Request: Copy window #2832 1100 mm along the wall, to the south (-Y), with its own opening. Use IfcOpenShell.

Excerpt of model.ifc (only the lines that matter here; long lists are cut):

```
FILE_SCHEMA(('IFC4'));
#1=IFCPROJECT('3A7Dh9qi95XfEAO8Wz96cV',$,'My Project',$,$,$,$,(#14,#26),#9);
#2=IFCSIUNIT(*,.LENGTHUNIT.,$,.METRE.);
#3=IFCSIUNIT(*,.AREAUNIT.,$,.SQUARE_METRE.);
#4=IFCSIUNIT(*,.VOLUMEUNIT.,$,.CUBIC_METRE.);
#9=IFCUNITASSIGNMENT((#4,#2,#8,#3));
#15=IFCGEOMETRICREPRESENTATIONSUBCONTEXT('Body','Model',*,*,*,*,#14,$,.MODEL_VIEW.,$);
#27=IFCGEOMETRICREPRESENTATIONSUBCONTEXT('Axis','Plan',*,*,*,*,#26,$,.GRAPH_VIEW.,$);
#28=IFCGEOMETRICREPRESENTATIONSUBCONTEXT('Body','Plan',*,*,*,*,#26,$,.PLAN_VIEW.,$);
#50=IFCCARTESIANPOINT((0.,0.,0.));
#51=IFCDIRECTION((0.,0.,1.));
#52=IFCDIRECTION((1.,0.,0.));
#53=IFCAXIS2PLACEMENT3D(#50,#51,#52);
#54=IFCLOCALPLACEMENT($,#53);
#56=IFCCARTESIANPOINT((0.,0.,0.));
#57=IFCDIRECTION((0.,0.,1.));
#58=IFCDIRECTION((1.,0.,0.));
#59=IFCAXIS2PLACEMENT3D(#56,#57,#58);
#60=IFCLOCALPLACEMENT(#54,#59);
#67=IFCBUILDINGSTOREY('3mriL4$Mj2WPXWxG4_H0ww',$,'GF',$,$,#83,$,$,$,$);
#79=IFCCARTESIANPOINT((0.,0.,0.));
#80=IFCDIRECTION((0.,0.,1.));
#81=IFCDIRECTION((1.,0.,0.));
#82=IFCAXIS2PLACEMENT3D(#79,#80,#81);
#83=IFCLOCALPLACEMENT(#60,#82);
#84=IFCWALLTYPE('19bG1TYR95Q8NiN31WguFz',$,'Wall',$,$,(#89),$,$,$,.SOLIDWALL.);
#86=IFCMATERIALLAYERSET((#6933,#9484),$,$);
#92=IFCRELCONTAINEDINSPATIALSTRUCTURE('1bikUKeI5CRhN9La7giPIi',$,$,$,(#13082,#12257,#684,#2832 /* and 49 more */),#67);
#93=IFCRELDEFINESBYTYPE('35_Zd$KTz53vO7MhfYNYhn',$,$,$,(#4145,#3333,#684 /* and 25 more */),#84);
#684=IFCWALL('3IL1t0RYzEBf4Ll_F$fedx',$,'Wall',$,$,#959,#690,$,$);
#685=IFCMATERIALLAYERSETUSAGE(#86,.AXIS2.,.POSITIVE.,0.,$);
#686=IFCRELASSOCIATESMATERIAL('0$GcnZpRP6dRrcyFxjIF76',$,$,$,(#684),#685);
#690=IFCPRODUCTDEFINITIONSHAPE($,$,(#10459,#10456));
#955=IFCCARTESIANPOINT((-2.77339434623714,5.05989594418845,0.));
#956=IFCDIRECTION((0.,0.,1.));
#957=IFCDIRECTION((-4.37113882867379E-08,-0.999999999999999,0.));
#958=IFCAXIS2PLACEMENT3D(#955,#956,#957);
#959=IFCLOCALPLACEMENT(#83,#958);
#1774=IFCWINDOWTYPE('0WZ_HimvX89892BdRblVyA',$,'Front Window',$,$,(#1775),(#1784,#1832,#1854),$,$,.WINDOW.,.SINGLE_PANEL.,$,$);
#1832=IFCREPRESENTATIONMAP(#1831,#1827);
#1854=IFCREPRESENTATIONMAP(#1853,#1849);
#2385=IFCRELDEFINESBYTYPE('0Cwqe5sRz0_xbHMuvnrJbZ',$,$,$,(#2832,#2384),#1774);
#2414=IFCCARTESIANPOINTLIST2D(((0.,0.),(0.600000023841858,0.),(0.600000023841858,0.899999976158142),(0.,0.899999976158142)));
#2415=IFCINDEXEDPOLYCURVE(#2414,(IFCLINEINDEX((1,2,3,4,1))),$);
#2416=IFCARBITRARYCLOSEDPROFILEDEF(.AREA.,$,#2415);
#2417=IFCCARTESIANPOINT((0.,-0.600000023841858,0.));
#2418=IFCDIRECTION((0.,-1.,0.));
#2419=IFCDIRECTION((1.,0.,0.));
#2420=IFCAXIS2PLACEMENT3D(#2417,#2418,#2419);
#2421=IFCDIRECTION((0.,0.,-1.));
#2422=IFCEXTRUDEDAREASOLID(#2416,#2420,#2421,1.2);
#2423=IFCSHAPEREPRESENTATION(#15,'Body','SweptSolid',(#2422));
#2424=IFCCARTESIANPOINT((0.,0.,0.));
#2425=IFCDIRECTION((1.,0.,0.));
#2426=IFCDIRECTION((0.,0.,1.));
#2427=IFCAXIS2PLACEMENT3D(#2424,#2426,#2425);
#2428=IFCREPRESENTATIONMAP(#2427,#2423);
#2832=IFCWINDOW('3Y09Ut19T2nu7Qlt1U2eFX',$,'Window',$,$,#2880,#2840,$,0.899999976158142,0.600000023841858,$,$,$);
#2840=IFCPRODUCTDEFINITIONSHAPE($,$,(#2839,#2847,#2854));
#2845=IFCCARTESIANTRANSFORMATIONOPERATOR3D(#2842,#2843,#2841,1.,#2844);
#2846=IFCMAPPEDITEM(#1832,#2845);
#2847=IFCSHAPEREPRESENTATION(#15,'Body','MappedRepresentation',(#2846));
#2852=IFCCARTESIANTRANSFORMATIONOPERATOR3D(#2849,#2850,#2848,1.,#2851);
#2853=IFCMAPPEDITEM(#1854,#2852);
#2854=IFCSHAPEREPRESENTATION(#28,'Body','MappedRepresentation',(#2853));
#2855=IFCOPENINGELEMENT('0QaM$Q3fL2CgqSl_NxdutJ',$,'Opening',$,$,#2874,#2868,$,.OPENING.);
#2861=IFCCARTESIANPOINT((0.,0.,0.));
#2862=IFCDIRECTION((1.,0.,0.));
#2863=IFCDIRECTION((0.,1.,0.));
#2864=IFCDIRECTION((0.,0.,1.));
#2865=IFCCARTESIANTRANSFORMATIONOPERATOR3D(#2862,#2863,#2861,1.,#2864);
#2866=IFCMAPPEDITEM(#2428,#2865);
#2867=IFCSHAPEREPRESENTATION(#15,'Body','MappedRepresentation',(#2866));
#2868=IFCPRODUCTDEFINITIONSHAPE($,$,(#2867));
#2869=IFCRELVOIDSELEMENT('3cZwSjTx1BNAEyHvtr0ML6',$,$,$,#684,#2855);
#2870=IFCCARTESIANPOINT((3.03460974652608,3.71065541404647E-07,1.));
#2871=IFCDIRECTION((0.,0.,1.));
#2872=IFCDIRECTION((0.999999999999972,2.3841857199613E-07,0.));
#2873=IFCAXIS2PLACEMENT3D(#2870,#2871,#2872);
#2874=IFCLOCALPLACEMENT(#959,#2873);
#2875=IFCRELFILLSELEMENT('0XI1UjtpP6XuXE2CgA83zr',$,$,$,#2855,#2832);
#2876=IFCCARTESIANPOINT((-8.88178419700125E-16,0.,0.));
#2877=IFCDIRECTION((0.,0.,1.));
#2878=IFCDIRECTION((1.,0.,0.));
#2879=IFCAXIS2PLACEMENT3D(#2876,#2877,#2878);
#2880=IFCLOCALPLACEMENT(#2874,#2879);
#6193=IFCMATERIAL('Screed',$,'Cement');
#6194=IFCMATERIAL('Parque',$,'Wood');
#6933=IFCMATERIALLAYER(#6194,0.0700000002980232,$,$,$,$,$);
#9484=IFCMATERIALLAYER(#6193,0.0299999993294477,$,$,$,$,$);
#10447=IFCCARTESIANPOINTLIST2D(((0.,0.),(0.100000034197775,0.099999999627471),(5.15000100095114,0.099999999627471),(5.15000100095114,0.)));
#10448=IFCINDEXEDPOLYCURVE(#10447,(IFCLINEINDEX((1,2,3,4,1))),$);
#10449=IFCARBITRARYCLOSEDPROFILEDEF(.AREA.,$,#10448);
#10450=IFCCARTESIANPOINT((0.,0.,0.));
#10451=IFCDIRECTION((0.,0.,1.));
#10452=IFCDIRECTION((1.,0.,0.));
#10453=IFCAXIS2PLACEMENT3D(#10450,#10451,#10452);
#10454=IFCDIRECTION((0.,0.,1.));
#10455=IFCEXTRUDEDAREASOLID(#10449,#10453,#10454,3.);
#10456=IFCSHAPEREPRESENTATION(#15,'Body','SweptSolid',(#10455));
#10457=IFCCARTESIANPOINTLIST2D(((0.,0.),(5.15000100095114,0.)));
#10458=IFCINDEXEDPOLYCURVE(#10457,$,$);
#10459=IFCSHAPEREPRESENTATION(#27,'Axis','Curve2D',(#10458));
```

```python
import ifcopenshell
import ifcopenshell.api.feature
import ifcopenshell.api.geometry
import ifcopenshell.api.root
import ifcopenshell.geom
import ifcopenshell.util.element
import ifcopenshell.util.placement
import ifcopenshell.util.shape

model = ifcopenshell.open("model.ifc")
settings = ifcopenshell.geom.settings()


def volume(element):
    """Net volume in cubic metres, openings subtracted."""
    shape = ifcopenshell.geom.create_shape(settings, element)
    return ifcopenshell.util.shape.get_volume(shape.geometry)


window = model.by_guid("3Y09Ut19T2nu7Qlt1U2eFX")
opening = window.FillsVoids[0].RelatingOpeningElement
wall = opening.VoidsElements[0].RelatingBuildingElement
before = volume(wall)
shift = ifcopenshell.util.placement.get_local_placement(wall.ObjectPlacement)[:3, 0] * 1.1

# copy_class copies the void relationship, type, container and properties, but no geometry.
new_opening = ifcopenshell.api.root.copy_class(model, product=opening)
new_opening.Representation = ifcopenshell.util.element.copy_deep(
    model, opening.Representation, exclude=["IfcGeometricRepresentationContext", "IfcRepresentationMap"]
)
new_window = ifcopenshell.api.root.copy_class(model, product=window)
new_window.Representation = ifcopenshell.util.element.copy_deep(
    model, window.Representation, exclude=["IfcGeometricRepresentationContext", "IfcRepresentationMap"]
)
ifcopenshell.api.feature.add_filling(model, opening=new_opening, element=new_window)

for old, new in ((opening, new_opening), (window, new_window)):
    matrix = ifcopenshell.util.placement.get_local_placement(old.ObjectPlacement)
    matrix[:3, 3] += shift
    ifcopenshell.api.geometry.edit_object_placement(model, product=new, matrix=matrix, is_si=False)

after = volume(wall)

print(f"wall volume {before:.3f} -> {after:.3f} m3")

model.write("model_v2.ifc")
```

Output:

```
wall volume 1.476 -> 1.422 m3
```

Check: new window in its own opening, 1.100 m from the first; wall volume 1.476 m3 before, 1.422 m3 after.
